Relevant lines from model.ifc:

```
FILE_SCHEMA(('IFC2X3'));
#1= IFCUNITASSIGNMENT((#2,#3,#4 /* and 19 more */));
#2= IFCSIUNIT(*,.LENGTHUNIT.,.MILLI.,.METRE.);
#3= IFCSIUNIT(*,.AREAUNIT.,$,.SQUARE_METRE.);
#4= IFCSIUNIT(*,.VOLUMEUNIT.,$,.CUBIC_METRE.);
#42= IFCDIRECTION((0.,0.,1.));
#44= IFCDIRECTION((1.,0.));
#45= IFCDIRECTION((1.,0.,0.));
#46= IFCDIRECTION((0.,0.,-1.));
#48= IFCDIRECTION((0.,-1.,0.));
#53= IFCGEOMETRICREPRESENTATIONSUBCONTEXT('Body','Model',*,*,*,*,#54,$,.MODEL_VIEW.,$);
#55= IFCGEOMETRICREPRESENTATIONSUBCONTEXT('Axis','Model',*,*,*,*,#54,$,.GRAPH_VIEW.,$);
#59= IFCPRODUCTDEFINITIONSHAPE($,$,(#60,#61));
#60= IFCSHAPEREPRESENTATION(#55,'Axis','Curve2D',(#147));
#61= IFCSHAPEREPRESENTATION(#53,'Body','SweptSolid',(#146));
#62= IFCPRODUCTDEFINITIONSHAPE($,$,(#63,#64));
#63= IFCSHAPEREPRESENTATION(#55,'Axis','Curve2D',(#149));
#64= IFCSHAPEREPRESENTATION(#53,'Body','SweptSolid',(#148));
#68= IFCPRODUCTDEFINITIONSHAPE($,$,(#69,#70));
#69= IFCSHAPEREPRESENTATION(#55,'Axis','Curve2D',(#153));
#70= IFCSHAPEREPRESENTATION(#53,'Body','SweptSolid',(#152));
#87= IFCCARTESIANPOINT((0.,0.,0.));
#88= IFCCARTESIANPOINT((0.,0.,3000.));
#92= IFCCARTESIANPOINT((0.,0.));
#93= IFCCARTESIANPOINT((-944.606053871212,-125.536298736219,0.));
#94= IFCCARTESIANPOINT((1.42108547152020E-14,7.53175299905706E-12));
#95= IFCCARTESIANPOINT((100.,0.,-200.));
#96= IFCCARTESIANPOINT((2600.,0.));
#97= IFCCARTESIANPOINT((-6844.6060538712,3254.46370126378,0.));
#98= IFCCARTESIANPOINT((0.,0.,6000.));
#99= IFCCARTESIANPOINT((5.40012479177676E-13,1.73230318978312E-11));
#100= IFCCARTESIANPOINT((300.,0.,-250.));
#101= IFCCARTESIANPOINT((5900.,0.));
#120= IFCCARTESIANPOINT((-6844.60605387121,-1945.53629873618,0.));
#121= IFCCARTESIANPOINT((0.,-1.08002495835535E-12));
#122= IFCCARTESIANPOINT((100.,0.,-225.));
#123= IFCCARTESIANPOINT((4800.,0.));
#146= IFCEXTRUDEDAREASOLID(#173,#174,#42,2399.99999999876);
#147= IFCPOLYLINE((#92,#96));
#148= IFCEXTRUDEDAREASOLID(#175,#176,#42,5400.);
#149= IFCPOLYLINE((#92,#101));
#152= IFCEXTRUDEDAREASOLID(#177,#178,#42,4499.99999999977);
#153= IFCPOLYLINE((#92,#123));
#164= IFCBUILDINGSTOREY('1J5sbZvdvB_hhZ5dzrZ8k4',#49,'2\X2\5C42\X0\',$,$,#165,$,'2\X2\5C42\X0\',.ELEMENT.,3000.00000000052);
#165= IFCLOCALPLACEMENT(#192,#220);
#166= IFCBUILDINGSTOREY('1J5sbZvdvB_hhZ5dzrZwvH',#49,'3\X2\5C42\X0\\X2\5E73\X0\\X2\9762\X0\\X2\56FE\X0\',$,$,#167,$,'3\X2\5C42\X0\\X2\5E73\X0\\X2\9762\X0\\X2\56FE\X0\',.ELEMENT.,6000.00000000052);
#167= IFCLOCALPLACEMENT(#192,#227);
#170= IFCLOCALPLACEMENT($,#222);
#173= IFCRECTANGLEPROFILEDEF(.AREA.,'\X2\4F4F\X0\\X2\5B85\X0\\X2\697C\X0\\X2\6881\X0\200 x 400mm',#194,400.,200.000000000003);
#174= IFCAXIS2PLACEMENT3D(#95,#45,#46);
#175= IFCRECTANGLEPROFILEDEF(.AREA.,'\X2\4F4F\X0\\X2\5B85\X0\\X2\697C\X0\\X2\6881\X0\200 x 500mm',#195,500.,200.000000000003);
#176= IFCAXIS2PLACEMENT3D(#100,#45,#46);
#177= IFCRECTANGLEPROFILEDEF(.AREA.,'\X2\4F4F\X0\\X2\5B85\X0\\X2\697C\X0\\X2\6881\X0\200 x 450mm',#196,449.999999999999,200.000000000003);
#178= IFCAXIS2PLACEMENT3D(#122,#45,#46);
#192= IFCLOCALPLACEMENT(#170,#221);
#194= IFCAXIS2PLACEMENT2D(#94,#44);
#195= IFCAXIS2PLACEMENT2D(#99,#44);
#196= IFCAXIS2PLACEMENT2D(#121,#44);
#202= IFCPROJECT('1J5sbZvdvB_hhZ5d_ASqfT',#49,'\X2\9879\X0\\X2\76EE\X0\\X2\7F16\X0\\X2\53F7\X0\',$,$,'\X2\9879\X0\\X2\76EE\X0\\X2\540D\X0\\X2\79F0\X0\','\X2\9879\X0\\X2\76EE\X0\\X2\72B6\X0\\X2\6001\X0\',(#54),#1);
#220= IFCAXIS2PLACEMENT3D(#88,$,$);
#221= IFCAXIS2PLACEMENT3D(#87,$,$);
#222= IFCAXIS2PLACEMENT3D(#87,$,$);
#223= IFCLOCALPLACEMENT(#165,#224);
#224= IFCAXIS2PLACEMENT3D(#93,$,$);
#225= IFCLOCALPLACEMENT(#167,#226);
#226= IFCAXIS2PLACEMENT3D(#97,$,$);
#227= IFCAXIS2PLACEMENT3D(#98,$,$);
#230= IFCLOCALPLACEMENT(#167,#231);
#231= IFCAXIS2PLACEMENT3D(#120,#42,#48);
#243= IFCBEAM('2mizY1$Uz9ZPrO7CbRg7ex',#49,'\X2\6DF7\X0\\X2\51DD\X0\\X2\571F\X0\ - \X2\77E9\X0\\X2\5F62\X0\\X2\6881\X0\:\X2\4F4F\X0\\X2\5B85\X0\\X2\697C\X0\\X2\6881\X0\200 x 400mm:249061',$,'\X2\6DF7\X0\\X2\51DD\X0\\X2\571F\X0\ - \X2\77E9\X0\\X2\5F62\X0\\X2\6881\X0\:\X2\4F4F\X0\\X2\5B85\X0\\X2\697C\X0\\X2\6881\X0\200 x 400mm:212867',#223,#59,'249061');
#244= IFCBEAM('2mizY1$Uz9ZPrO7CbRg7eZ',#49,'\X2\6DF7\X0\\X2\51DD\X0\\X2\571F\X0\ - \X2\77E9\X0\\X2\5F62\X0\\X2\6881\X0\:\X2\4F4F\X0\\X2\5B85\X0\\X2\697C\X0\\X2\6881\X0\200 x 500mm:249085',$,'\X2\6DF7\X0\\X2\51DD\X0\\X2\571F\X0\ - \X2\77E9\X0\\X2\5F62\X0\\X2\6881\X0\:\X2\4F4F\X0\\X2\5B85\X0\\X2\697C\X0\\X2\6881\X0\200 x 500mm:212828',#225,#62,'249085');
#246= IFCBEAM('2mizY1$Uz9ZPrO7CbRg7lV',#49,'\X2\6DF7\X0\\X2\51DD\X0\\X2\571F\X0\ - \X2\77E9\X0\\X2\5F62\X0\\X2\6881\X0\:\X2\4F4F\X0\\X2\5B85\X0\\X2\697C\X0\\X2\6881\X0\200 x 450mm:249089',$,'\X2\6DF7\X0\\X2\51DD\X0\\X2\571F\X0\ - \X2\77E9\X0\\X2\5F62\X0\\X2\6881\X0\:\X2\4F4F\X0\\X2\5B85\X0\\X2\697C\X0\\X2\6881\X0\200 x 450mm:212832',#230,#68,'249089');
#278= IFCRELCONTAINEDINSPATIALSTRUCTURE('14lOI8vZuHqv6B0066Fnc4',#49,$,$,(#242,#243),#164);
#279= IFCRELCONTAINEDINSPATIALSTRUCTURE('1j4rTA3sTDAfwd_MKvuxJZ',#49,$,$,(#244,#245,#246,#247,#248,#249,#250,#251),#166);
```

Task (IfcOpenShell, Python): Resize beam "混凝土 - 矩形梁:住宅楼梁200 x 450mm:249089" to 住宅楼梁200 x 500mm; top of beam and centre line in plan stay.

```python
import ifcopenshell
import ifcopenshell.util.element
import ifcopenshell.util.representation

model = ifcopenshell.open("model.ifc")

member = model.by_id(246)
source = next(p for p in model.by_type("IfcRectangleProfileDef") if p.ProfileName == "住宅楼梁200 x 500mm")

body = ifcopenshell.util.representation.get_representation(member, "Model", "Body")
solid = body.Items[0]
old_profile = solid.SweptArea

# Copy the section's sizes but keep this member's own profile position.
profile = ifcopenshell.util.element.copy(model, source)
# Profiles are centred, so shift by half the change in depth to hold the top.
shift = (old_profile.XDim - profile.XDim) / 2
x, y = old_profile.Position.Location.Coordinates
up = (-1.0, 0.0)  # upwards, in the solid's own plane
location = model.createIfcCartesianPoint((x + up[0] * shift, y + up[1] * shift))
profile.Position = model.createIfcAxis2Placement2D(location, old_profile.Position.RefDirection)
solid.SweptArea = profile
if not model.get_total_inverses(old_profile):
    ifcopenshell.util.element.remove_deep2(model, old_profile)
member.Name = member.Name.replace("住宅楼梁200 x 450mm", "住宅楼梁200 x 500mm")
member.ObjectType = member.ObjectType.replace("住宅楼梁200 x 450mm", "住宅楼梁200 x 500mm")

print(solid.SweptArea)

model.write("model_edited.ifc")
```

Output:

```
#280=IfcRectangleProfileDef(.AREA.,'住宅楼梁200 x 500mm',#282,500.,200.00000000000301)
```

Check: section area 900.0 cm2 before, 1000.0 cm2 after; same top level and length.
